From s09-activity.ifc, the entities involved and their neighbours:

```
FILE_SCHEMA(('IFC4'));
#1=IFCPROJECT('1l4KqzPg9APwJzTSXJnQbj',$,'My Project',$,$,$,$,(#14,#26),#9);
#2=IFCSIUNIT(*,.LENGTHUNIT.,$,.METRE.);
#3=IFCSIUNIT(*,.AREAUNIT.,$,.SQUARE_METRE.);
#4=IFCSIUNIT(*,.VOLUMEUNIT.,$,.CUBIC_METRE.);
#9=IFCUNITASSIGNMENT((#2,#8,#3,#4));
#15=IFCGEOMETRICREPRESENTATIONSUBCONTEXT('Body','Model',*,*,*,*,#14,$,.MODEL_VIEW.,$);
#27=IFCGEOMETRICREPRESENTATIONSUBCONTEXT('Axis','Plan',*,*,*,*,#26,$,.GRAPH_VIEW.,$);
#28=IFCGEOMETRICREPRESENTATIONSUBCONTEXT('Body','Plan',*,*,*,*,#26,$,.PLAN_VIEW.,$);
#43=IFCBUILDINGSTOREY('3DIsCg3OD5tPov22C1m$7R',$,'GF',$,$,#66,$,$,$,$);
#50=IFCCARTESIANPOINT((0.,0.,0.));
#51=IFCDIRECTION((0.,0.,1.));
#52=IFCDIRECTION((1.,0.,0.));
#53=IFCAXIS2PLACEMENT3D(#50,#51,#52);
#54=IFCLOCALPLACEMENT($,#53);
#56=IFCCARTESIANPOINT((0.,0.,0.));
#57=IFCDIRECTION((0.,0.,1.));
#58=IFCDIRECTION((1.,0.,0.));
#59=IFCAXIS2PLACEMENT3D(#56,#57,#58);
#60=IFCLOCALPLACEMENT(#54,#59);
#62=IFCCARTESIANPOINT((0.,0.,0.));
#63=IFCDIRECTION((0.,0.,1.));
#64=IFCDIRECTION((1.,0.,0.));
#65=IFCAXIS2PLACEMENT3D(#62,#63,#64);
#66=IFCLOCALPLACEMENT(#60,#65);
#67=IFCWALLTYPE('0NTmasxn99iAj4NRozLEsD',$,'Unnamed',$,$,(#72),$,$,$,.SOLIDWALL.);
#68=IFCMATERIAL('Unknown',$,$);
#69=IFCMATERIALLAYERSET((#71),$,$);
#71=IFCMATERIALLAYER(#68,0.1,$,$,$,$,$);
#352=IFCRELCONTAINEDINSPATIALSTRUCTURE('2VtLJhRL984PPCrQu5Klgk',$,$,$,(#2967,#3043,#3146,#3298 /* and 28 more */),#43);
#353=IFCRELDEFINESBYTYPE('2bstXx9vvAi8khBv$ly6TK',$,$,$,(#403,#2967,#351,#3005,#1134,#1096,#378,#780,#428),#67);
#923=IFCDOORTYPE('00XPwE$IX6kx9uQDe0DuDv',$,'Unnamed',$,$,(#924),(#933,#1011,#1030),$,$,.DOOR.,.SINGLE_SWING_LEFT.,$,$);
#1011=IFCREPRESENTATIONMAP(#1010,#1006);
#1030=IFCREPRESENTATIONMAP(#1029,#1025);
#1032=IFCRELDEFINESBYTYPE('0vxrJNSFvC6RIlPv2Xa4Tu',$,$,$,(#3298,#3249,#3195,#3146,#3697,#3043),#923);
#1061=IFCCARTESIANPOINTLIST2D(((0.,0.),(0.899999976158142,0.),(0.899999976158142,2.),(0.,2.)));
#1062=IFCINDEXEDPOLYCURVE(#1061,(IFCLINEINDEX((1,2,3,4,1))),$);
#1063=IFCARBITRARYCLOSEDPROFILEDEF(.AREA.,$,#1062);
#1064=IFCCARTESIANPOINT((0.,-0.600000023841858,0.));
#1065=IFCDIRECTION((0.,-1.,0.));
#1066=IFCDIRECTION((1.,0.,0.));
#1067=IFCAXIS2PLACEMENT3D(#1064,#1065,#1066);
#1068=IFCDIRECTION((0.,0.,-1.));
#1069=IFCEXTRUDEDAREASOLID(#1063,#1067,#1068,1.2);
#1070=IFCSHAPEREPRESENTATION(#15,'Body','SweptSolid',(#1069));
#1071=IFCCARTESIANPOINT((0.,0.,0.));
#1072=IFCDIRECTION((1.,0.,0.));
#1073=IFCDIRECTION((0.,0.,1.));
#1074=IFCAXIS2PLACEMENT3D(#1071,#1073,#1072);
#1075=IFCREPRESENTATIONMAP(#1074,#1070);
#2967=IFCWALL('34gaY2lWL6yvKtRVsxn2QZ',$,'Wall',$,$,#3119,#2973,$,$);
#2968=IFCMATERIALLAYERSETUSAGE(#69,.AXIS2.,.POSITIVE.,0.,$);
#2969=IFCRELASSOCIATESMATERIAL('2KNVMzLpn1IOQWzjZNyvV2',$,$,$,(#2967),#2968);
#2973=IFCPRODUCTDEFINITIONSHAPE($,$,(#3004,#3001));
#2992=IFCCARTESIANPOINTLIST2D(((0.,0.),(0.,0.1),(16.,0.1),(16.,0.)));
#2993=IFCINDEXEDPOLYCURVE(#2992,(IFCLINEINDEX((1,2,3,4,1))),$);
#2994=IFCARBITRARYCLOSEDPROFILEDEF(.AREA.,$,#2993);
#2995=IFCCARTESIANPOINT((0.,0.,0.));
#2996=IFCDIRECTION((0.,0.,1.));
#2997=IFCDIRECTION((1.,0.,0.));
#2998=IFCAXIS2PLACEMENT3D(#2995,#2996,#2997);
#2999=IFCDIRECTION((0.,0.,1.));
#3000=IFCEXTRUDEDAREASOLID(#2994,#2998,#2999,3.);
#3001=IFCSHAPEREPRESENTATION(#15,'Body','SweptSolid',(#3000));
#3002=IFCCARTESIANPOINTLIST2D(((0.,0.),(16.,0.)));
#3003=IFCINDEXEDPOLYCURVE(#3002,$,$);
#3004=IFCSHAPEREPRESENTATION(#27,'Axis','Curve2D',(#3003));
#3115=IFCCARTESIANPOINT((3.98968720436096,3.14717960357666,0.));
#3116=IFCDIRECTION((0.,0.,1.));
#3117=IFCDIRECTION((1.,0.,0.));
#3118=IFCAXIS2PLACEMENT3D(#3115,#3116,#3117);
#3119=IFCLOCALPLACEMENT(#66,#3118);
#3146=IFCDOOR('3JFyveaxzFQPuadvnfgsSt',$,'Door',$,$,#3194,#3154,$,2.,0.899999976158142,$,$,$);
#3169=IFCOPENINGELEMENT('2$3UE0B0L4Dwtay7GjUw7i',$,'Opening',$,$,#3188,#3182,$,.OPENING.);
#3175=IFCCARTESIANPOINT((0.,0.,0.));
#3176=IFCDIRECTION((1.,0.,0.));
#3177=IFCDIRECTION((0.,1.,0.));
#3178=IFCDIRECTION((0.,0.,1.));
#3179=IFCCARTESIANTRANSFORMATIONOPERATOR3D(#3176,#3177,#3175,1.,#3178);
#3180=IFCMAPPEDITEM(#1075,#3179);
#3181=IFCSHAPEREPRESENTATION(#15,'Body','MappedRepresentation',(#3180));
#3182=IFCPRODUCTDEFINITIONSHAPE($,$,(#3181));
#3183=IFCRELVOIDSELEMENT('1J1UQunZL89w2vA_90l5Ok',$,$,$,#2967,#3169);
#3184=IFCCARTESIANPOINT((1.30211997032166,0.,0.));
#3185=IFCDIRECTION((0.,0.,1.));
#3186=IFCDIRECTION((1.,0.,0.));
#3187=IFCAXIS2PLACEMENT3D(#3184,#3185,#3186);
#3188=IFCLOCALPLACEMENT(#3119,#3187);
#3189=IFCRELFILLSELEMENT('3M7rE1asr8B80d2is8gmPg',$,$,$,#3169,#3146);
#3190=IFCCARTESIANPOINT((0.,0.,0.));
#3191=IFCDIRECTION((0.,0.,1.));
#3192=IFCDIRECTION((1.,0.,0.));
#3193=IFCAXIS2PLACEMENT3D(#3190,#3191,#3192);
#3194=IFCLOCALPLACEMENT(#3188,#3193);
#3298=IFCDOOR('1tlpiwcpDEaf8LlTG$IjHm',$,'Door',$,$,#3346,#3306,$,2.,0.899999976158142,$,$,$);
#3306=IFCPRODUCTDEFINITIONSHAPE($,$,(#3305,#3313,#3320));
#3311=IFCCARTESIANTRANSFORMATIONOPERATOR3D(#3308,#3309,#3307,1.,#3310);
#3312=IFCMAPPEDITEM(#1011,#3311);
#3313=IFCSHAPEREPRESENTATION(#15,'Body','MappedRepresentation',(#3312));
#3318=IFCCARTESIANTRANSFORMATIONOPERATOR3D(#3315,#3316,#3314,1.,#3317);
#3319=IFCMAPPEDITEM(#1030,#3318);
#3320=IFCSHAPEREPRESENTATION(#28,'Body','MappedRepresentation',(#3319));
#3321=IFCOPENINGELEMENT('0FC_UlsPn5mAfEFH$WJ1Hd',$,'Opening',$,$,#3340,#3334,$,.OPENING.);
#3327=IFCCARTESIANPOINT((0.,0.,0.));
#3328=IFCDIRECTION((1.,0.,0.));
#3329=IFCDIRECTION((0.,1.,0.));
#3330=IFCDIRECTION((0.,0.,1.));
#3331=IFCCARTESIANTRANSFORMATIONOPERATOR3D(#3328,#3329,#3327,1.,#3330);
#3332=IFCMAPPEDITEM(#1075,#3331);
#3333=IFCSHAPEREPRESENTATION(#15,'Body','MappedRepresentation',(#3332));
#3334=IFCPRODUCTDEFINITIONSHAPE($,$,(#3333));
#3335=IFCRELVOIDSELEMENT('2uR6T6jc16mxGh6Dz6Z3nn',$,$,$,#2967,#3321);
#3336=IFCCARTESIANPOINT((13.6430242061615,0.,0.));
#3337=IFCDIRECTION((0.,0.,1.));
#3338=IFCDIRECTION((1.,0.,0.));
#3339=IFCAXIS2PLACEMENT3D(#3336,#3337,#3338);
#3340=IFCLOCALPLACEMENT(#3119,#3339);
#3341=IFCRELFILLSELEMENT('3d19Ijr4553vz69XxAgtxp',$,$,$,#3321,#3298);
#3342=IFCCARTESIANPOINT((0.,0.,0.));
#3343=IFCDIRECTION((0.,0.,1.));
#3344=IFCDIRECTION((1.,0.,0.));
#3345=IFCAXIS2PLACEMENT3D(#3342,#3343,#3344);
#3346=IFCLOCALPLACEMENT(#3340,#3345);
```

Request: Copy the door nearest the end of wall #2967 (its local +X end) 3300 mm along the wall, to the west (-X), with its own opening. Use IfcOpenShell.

```python
import ifcopenshell
import ifcopenshell.api.feature
import ifcopenshell.api.geometry
import ifcopenshell.api.root
import ifcopenshell.geom
import ifcopenshell.util.element
import ifcopenshell.util.placement
import ifcopenshell.util.shape
import ifcopenshell.util.unit

model = ifcopenshell.open("s09-activity.ifc")
unit_scale = ifcopenshell.util.unit.calculate_unit_scale(model)
settings = ifcopenshell.geom.settings()


def volume(element):
    """Net volume in cubic metres, openings subtracted."""
    shape = ifcopenshell.geom.create_shape(settings, element)
    return ifcopenshell.util.shape.get_volume(shape.geometry)


door = model.by_guid("1tlpiwcpDEaf8LlTG$IjHm")
opening = door.FillsVoids[0].RelatingOpeningElement
wall = opening.VoidsElements[0].RelatingBuildingElement
before = volume(wall)
shift = ifcopenshell.util.placement.get_local_placement(wall.ObjectPlacement)[:3, 0] * -3.3 / unit_scale

# copy_class copies the void relationship, type, container and properties, but no geometry.
new_opening = ifcopenshell.api.root.copy_class(model, product=opening)
new_opening.Representation = ifcopenshell.util.element.copy_deep(
    model, opening.Representation, exclude=["IfcGeometricRepresentationContext", "IfcRepresentationMap"]
)
new_door = ifcopenshell.api.root.copy_class(model, product=door)
new_door.Representation = ifcopenshell.util.element.copy_deep(
    model, door.Representation, exclude=["IfcGeometricRepresentationContext", "IfcRepresentationMap"]
)
ifcopenshell.api.feature.add_filling(model, opening=new_opening, element=new_door)

for old, new in ((opening, new_opening), (door, new_door)):
    matrix = ifcopenshell.util.placement.get_local_placement(old.ObjectPlacement)
    matrix[:3, 3] += shift
    ifcopenshell.api.geometry.edit_object_placement(model, product=new, matrix=matrix, is_si=False)

after = volume(wall)

print(f"wall volume {before:.3f} -> {after:.3f} m3")

model.write("s09-activity-out.ifc")
```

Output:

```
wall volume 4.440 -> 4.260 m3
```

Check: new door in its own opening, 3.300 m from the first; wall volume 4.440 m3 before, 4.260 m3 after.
